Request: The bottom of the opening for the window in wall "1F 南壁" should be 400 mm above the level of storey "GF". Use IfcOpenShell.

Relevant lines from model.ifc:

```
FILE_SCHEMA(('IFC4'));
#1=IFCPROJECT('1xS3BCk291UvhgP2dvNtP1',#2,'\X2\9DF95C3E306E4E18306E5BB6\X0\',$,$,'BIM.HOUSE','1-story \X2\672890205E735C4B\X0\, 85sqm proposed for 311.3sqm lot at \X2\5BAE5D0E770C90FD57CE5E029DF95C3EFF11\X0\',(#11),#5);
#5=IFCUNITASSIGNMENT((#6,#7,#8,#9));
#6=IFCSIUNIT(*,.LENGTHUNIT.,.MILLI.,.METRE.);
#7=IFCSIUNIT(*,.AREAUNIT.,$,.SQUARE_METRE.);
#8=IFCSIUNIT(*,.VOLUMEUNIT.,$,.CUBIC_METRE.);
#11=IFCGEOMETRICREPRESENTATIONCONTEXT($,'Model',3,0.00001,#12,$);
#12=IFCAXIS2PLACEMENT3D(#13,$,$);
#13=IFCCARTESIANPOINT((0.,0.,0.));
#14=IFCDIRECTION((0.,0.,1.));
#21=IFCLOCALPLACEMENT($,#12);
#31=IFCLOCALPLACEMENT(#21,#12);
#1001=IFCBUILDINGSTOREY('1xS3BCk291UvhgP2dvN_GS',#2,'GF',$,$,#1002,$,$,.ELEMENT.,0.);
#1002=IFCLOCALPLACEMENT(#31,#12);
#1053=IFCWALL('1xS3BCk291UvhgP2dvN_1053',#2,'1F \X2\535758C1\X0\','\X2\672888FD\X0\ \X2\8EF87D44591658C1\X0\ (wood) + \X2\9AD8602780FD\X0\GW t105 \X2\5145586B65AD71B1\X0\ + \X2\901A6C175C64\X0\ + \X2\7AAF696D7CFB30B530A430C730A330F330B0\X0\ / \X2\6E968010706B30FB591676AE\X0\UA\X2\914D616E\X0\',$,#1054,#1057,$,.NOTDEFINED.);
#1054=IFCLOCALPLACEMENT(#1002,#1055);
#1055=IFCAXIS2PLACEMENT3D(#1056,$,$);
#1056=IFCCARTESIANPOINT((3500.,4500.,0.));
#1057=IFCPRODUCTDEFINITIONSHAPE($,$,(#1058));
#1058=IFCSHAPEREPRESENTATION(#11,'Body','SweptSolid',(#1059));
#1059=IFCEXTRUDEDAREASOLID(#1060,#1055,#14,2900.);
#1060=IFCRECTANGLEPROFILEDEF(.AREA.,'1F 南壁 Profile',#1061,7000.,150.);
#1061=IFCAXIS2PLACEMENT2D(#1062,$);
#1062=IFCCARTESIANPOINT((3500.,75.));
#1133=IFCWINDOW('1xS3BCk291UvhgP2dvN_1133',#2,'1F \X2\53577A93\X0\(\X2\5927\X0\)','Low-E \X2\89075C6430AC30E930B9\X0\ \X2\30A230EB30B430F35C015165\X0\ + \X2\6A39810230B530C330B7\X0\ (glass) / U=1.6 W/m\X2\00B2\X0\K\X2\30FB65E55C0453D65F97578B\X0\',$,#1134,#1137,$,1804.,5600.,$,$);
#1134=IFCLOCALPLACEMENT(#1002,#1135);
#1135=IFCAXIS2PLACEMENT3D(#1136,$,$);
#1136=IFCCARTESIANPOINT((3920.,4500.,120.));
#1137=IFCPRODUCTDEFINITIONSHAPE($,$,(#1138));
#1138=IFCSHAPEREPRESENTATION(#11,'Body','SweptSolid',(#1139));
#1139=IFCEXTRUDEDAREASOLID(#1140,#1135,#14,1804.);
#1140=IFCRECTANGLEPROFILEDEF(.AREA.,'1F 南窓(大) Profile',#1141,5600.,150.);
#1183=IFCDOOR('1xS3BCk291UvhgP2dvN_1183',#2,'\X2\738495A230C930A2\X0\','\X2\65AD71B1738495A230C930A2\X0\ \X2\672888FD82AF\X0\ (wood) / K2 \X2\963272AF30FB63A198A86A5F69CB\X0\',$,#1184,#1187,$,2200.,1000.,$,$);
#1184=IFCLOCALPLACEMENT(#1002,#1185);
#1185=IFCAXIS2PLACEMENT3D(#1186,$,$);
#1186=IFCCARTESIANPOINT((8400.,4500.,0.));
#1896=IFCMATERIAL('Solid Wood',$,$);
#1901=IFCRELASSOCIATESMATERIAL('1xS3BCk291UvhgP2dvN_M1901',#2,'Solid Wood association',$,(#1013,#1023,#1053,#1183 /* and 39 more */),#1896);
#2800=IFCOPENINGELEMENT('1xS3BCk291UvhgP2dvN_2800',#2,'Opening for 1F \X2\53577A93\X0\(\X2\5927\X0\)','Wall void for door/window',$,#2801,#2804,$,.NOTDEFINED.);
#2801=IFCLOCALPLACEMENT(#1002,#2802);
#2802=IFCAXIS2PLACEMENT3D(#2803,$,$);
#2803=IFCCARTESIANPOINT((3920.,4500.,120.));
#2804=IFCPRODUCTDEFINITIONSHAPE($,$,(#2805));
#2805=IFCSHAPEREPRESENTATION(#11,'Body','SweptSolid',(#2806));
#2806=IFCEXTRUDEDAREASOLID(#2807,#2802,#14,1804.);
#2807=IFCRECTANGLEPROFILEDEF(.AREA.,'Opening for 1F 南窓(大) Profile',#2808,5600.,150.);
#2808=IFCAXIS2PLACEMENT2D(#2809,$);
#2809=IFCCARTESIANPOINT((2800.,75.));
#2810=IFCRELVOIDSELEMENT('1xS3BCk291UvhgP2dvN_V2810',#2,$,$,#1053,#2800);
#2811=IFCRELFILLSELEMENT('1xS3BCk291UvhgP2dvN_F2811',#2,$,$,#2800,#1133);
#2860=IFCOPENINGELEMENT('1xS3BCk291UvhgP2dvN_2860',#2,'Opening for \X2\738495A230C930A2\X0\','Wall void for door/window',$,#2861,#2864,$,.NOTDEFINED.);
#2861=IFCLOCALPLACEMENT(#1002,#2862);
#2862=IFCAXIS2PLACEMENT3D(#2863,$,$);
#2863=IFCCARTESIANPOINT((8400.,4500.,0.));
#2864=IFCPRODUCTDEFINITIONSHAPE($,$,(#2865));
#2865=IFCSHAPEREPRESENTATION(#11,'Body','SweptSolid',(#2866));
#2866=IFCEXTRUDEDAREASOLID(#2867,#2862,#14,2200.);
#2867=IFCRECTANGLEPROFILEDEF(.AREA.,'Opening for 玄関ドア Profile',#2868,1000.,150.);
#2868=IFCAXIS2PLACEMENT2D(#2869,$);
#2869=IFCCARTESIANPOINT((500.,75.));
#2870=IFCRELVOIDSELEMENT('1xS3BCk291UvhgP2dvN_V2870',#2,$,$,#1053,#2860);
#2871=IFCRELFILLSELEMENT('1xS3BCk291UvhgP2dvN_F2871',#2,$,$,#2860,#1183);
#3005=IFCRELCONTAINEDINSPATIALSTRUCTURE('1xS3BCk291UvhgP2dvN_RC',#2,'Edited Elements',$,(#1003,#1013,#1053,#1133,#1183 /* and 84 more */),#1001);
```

```python
import numpy as np
import ifcopenshell
import ifcopenshell.api.geometry
import ifcopenshell.geom
import ifcopenshell.util.element
import ifcopenshell.util.placement
import ifcopenshell.util.shape
import ifcopenshell.util.unit

model = ifcopenshell.open("model.ifc")
unit_scale = ifcopenshell.util.unit.calculate_unit_scale(model)

window = model.by_id(1133)
opening = window.FillsVoids[0].RelatingOpeningElement
storey = ifcopenshell.util.element.get_container(window, ifc_class="IfcBuildingStorey")
level = ifcopenshell.util.placement.get_local_placement(storey.ObjectPlacement)[2, 3]

# The opening's origin need not be at the sill, so measure its lowest point.
shape = ifcopenshell.geom.create_shape(ifcopenshell.geom.settings(), opening)
bottom = ifcopenshell.util.shape.get_shape_bottom_elevation(shape, shape.geometry) / unit_scale
dz = level + 400.0 - bottom

shift = np.array([0.0, 0.0, dz])
# The window is not placed relative to its opening, so move both.
for product in (opening, window):
    matrix = ifcopenshell.util.placement.get_local_placement(product.ObjectPlacement)
    matrix[:3, 3] += shift
    ifcopenshell.api.geometry.edit_object_placement(model, product=product, matrix=matrix, is_si=False)

print(f"moved by {dz * unit_scale:+.3f} m")

model.write("model_rev.ifc")
```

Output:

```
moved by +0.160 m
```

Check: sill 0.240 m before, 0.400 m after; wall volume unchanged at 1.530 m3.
